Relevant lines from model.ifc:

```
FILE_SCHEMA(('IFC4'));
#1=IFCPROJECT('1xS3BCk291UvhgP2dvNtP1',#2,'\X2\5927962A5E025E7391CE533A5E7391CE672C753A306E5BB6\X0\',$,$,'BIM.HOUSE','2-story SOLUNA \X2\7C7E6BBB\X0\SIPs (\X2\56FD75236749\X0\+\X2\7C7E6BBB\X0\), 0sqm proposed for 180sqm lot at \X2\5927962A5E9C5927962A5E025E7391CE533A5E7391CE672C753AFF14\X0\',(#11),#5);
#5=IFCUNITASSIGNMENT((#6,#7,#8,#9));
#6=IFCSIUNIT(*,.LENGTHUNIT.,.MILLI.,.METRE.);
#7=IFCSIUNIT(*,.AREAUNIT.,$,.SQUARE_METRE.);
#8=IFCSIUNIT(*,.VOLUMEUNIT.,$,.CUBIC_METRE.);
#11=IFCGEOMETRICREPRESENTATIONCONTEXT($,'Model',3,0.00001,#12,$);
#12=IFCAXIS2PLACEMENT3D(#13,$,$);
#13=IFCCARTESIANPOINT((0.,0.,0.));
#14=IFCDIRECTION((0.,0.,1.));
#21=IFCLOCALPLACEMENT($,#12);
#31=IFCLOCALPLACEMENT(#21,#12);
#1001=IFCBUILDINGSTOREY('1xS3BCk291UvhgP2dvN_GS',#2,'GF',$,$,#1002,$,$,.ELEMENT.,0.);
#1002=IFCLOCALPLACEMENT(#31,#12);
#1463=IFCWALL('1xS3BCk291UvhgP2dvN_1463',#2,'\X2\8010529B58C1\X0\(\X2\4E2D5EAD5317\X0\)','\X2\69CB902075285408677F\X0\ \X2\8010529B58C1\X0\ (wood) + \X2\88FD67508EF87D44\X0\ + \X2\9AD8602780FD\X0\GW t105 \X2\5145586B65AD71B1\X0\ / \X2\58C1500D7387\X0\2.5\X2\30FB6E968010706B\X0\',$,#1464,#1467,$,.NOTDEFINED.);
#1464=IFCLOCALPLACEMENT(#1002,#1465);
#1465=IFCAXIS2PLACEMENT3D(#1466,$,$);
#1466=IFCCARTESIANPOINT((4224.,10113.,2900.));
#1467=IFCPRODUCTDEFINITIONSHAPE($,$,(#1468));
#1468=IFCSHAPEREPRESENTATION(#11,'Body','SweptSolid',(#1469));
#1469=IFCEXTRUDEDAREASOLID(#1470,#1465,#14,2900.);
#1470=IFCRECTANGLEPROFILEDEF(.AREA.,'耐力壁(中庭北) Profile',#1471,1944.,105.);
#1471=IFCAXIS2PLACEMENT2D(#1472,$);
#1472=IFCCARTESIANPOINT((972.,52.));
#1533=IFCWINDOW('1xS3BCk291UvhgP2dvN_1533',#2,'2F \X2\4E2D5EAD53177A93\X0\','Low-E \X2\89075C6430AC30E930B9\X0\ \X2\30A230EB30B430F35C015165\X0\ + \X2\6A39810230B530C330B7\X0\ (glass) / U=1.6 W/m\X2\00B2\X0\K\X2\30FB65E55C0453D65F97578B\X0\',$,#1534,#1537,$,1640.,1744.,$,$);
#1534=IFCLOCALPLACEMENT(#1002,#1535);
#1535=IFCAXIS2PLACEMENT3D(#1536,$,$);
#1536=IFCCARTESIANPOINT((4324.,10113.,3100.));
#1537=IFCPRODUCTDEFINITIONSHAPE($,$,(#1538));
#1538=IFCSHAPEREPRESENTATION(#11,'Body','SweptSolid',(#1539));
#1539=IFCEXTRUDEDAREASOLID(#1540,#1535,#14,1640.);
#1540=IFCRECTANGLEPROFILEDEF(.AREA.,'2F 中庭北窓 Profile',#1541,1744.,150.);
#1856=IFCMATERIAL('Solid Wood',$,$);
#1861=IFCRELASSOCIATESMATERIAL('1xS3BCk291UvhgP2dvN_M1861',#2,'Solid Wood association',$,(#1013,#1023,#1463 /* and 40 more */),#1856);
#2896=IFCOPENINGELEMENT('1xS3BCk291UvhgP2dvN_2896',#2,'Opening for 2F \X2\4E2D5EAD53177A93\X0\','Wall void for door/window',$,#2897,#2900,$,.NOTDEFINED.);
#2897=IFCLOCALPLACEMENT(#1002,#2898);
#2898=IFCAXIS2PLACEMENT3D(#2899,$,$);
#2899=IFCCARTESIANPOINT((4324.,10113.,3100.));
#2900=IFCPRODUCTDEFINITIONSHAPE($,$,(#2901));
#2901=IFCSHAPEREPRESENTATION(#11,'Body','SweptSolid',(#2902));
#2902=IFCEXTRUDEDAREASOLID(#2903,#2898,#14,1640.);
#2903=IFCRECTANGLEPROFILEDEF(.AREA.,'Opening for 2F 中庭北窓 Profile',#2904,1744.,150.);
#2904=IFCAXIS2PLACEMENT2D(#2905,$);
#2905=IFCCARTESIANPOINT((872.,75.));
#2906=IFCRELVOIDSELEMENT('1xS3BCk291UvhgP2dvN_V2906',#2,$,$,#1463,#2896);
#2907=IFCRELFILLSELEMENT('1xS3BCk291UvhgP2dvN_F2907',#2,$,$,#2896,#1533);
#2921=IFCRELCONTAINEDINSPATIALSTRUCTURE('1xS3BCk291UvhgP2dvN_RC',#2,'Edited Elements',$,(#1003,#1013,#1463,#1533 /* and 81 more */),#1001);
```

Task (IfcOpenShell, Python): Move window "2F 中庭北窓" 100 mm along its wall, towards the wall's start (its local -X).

```python
import ifcopenshell
import ifcopenshell.api.geometry
import ifcopenshell.util.placement
import ifcopenshell.util.unit

model = ifcopenshell.open("model.ifc")
unit_scale = ifcopenshell.util.unit.calculate_unit_scale(model)

window = model.by_guid("1xS3BCk291UvhgP2dvN_1533")
opening = window.FillsVoids[0].RelatingOpeningElement
wall = opening.VoidsElements[0].RelatingBuildingElement

wall_matrix = ifcopenshell.util.placement.get_local_placement(wall.ObjectPlacement)
shift = wall_matrix[:3, 0] * -0.1 / unit_scale
before = ifcopenshell.util.placement.get_local_placement(window.ObjectPlacement)[:3, 3].copy()

# The window is not placed relative to its opening, so move both.
for product in (opening, window):
    matrix = ifcopenshell.util.placement.get_local_placement(product.ObjectPlacement)
    matrix[:3, 3] += shift
    ifcopenshell.api.geometry.edit_object_placement(model, product=product, matrix=matrix, is_si=False)

after = ifcopenshell.util.placement.get_local_placement(window.ObjectPlacement)[:3, 3]
print("window moved by", (after - before).round(3) + 0.0)

model.write("model_edited.ifc")
```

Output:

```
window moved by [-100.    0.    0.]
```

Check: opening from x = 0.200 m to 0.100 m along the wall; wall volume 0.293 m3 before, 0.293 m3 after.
